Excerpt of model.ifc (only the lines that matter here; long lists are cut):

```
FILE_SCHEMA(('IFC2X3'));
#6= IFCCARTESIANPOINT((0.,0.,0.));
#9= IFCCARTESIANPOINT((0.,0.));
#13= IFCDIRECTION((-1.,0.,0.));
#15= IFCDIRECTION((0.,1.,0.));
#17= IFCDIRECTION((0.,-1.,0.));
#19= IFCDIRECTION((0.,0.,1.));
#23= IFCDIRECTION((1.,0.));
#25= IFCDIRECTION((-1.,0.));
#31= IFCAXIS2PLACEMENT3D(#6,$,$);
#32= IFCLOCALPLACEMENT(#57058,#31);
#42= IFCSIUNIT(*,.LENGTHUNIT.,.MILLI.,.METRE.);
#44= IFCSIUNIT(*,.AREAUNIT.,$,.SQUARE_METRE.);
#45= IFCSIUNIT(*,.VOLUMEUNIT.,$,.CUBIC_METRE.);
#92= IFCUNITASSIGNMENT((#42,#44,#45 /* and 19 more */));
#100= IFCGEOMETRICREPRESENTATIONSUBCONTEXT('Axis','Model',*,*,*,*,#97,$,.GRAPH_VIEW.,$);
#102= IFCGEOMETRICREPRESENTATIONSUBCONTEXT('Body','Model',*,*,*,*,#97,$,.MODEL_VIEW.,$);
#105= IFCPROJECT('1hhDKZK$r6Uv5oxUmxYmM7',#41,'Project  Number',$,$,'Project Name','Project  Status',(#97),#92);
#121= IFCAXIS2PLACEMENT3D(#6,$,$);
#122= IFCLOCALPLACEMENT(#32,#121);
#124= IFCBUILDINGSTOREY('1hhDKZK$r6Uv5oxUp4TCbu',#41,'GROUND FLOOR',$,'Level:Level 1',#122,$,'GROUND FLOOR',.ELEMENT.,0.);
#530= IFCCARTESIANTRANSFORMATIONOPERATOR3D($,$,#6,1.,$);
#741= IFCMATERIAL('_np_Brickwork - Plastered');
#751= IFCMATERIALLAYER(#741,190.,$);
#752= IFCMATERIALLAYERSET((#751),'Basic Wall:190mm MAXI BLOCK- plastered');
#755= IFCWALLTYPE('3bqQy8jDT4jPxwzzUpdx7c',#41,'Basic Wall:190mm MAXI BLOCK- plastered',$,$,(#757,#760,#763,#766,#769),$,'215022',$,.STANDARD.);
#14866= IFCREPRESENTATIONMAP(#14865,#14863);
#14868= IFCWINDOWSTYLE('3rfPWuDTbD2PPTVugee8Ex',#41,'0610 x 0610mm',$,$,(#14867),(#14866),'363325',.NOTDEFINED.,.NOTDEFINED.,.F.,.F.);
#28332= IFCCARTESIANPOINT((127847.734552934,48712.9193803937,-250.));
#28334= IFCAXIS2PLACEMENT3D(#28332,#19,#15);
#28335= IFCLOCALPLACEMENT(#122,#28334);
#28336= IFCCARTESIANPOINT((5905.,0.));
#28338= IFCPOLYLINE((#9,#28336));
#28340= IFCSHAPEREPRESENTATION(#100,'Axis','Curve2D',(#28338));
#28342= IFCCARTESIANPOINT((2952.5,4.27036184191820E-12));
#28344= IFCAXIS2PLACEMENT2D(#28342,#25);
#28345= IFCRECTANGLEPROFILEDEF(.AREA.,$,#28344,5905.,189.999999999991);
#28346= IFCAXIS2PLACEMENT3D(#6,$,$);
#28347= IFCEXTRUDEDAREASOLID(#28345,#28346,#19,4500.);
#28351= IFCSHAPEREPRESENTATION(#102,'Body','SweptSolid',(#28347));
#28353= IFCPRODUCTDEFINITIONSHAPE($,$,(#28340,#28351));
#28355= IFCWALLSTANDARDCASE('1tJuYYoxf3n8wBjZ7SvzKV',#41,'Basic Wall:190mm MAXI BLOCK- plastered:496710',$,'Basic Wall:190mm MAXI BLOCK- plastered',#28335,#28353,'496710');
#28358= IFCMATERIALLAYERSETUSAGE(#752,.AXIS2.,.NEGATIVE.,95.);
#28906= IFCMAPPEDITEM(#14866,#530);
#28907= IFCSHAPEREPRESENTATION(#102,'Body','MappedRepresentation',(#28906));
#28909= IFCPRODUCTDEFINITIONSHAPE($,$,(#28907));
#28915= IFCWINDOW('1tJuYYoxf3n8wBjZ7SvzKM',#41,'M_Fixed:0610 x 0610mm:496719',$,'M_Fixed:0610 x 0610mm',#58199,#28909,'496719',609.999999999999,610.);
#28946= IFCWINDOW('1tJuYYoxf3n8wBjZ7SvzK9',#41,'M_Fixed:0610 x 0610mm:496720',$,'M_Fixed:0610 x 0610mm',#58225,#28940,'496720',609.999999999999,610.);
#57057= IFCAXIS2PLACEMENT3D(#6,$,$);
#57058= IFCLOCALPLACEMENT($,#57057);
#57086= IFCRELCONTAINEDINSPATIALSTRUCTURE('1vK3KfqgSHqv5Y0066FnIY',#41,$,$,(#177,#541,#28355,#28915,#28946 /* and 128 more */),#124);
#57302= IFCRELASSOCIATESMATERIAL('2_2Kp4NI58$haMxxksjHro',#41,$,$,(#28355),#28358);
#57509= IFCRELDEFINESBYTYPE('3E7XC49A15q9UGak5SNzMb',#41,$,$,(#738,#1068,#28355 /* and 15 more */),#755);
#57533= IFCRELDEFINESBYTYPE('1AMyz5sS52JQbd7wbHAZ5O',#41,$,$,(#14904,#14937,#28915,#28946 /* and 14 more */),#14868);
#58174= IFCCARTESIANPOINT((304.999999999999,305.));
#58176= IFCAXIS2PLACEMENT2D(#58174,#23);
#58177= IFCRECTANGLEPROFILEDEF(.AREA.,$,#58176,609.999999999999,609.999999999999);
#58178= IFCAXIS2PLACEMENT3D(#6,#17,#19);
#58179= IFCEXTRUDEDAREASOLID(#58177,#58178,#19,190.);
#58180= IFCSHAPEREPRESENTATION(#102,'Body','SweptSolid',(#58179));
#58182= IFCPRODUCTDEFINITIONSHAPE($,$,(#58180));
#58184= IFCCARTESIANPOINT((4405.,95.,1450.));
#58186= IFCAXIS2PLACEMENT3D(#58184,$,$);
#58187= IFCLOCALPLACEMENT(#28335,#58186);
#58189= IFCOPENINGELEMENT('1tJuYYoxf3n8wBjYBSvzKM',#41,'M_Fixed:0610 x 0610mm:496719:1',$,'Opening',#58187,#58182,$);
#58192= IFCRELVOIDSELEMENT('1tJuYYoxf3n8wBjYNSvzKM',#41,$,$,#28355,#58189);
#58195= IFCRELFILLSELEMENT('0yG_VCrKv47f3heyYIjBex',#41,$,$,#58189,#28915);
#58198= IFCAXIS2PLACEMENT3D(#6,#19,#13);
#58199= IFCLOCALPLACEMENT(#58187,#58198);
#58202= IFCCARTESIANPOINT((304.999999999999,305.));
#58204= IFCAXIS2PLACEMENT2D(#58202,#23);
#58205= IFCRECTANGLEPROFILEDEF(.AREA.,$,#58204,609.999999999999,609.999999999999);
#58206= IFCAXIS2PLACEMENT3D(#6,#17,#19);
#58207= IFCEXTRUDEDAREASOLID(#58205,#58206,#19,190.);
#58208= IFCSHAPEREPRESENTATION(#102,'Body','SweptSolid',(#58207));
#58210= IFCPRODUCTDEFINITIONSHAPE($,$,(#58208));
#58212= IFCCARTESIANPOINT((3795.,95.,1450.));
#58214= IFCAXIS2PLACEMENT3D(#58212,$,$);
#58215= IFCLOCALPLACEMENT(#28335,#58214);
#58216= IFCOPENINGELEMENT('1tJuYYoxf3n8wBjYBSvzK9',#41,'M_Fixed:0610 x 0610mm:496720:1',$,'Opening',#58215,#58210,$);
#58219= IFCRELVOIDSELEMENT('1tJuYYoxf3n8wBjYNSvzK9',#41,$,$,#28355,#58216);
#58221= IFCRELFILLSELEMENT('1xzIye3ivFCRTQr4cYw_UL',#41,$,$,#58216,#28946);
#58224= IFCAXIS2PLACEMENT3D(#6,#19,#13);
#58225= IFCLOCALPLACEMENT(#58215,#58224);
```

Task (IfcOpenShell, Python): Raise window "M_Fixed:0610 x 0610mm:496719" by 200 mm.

```python
import numpy as np
import ifcopenshell
import ifcopenshell.api.geometry
import ifcopenshell.util.placement
import ifcopenshell.util.unit

model = ifcopenshell.open("model.ifc")
unit_scale = ifcopenshell.util.unit.calculate_unit_scale(model)

window = model.by_guid("1tJuYYoxf3n8wBjZ7SvzKM")
opening = window.FillsVoids[0].RelatingOpeningElement
dz = 0.2 / unit_scale

shift = np.array([0.0, 0.0, dz])
# The window is placed relative to its opening, so it follows when the opening moves.
matrix = ifcopenshell.util.placement.get_local_placement(opening.ObjectPlacement)
matrix[:3, 3] += shift
ifcopenshell.api.geometry.edit_object_placement(
    model, product=opening, matrix=matrix, is_si=False, should_transform_children=True
)

print(f"moved by {dz * unit_scale:+.3f} m")

model.write("model-out.ifc")
```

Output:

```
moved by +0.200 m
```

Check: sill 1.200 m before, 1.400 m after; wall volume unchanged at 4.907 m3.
